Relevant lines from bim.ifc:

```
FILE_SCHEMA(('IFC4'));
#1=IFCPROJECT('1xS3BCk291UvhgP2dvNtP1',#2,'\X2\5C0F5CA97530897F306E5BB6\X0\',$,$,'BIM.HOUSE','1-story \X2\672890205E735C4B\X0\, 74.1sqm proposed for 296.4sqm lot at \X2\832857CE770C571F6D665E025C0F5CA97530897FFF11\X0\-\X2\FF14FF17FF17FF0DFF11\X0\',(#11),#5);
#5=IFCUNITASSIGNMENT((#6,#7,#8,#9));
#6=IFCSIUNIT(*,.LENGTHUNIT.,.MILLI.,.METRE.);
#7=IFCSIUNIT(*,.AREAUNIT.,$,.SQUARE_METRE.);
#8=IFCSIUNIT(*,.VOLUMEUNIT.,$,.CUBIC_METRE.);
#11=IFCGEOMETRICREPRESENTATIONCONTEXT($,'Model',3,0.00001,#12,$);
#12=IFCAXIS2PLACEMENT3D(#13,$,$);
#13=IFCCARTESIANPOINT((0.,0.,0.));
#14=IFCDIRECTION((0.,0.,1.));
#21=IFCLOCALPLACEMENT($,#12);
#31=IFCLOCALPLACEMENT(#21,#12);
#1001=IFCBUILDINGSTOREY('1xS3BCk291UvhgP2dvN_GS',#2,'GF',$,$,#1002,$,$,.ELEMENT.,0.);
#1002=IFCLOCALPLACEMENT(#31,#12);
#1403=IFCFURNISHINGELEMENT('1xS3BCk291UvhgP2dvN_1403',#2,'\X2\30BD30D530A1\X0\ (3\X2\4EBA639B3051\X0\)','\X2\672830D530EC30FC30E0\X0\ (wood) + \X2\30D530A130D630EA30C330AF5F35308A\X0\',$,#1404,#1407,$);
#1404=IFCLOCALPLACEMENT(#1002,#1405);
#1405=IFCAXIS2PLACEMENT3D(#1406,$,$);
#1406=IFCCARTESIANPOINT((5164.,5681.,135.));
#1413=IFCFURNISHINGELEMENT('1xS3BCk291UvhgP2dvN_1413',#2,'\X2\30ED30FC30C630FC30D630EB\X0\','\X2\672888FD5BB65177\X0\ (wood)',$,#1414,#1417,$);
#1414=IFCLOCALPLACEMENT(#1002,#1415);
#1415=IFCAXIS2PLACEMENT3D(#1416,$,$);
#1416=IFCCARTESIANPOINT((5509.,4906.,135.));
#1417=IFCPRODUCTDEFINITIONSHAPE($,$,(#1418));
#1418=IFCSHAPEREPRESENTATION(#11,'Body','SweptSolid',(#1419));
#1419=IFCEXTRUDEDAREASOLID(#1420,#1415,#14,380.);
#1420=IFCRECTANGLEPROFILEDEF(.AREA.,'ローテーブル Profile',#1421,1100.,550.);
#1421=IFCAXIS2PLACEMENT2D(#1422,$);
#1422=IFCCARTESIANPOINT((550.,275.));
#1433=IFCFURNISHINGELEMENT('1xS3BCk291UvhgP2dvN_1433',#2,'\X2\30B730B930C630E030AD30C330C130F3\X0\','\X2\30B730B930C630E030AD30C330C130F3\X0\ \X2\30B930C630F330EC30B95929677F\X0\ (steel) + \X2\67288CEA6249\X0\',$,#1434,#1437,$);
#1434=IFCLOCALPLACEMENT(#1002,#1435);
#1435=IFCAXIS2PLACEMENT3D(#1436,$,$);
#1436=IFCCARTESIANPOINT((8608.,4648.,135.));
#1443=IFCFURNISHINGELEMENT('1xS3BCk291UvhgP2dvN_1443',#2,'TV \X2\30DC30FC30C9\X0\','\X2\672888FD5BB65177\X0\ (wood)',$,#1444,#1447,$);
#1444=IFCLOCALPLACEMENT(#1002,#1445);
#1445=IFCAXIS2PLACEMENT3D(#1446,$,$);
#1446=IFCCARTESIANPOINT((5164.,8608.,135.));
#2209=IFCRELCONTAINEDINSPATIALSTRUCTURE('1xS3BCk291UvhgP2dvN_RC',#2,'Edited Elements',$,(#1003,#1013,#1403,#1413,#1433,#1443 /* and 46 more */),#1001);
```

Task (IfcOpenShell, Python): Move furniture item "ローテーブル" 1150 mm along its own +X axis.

```python
import ifcopenshell
import ifcopenshell.api.geometry
import ifcopenshell.util.placement
import ifcopenshell.util.unit

model = ifcopenshell.open("bim.ifc")
unit_scale = ifcopenshell.util.unit.calculate_unit_scale(model)

item = model.by_guid("1xS3BCk291UvhgP2dvN_1413")
matrix = ifcopenshell.util.placement.get_local_placement(item.ObjectPlacement)
matrix[:3, 3] += matrix[:3, 0] * 1.15 / unit_scale
ifcopenshell.api.geometry.edit_object_placement(model, product=item, matrix=matrix, is_si=False)

print(ifcopenshell.util.placement.get_local_placement(item.ObjectPlacement).round(3) + 0.0)

model.write("bim-out.ifc")
```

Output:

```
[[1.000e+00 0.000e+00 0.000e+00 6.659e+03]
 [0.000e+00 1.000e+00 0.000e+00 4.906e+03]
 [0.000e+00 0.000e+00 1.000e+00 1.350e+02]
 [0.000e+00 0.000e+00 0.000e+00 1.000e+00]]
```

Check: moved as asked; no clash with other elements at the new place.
